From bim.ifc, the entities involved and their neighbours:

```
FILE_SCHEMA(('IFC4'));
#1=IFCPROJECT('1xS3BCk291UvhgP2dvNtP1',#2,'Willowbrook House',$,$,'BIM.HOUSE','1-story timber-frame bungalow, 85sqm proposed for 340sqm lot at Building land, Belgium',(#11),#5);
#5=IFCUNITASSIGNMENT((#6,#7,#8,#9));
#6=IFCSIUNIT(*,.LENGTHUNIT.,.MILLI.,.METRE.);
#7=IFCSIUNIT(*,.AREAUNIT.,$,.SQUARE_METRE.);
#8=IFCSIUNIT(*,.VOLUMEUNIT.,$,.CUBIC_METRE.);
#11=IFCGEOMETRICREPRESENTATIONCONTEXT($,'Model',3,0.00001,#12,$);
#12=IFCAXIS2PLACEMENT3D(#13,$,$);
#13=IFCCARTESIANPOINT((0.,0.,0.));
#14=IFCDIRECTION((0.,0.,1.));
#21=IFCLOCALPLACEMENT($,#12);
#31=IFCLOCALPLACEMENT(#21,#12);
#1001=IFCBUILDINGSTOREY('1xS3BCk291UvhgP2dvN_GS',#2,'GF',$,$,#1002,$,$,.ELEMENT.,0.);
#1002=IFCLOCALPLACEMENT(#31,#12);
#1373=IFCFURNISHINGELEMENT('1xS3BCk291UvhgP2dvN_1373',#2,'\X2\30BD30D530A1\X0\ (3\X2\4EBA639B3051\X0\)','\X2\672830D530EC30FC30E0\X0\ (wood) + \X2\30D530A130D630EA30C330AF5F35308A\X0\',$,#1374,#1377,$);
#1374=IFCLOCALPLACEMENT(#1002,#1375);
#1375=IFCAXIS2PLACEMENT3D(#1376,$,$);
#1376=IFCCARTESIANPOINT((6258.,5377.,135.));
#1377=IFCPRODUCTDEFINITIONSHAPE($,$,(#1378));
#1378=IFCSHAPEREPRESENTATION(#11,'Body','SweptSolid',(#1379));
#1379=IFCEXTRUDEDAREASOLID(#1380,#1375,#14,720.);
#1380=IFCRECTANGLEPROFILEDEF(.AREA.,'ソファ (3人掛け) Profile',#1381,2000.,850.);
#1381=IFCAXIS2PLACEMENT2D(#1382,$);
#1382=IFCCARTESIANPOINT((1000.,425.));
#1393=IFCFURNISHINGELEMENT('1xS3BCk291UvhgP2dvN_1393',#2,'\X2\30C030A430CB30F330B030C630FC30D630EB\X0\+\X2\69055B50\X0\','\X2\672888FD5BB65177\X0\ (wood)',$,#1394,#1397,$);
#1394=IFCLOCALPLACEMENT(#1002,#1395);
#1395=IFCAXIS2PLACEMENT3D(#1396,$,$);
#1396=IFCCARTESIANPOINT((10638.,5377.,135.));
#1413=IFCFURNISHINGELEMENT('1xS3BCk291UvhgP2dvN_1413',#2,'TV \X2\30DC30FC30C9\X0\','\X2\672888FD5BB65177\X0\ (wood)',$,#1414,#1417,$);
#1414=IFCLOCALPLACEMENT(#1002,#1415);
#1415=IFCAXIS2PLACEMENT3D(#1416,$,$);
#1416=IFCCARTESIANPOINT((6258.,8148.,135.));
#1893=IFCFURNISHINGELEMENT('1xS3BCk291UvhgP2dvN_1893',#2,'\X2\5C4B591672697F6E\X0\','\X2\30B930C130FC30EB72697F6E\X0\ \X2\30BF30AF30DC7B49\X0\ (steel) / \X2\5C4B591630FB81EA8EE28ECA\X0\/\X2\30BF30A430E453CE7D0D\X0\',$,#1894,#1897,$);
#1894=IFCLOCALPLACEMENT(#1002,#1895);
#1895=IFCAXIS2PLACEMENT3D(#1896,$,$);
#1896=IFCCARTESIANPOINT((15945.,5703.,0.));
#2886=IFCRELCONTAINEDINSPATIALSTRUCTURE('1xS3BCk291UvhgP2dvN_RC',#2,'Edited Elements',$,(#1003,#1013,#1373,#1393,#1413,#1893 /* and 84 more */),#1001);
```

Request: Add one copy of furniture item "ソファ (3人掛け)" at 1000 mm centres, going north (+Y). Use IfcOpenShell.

```python
import numpy as np
import ifcopenshell
import ifcopenshell.api.geometry
import ifcopenshell.api.root
import ifcopenshell.util.element
import ifcopenshell.util.placement
import ifcopenshell.util.unit

model = ifcopenshell.open("bim.ifc")
unit_scale = ifcopenshell.util.unit.calculate_unit_scale(model)


def reuse_history(source, copy):
    """copy_class also copies each property set's owner history, people and application; keep the originals."""
    for rel in copy.IsDefinedBy:
        if rel.is_a("IfcRelDefinesByProperties") and (history := rel.RelatingPropertyDefinition.OwnerHistory):
            rel.RelatingPropertyDefinition.OwnerHistory = source.OwnerHistory
            ifcopenshell.util.element.remove_deep2(model, history)


source = model.by_guid("1xS3BCk291UvhgP2dvN_1373")
base = ifcopenshell.util.placement.get_local_placement(source.ObjectPlacement)
step = np.array([0.0, 1.0, 0.0]) * 1 / unit_scale

for i in range(1, 2):
    copy = ifcopenshell.api.root.copy_class(model, product=source)
    copy.Representation = ifcopenshell.util.element.copy_deep(
        model, source.Representation, exclude=["IfcGeometricRepresentationContext", "IfcRepresentationMap"]
    )
    reuse_history(source, copy)
    matrix = base.copy()
    matrix[:3, 3] += i * step
    print("added at", matrix[:3, 3].round(3) + 0.0)
    ifcopenshell.api.geometry.edit_object_placement(model, product=copy, matrix=matrix, is_si=False)

model.write("bim_updated.ifc")
```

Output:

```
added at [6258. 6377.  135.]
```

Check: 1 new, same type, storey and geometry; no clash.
